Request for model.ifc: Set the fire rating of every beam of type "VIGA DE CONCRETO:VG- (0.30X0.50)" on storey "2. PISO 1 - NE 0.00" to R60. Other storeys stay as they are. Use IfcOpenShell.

First a look at what the model holds.

```python
import ifcopenshell
import ifcopenshell.util.element

model = ifcopenshell.open("model.ifc")
print(model.schema)
storey = next(s for s in model.by_type("IfcBuildingStorey") if s.Name == "2. PISO 1 - NE 0.00")
beams = [e for e in ifcopenshell.util.element.get_decomposition(storey) if e.is_a("IfcBeam")]
seen = {}
for e in beams:
    element_type = ifcopenshell.util.element.get_type(e)
    key = (element_type.Name if element_type != e and element_type else None, ifcopenshell.util.element.get_pset(e, "Pset_BeamCommon", "FireRating"))
    seen[key] = seen.get(key, 0) + 1
for (name, value), count in sorted(seen.items(), key=str):
    print(count, "x", name, "|", value)
```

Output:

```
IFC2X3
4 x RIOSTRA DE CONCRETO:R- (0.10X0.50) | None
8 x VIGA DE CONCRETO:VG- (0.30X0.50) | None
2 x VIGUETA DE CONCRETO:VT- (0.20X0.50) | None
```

```python
import ifcopenshell
import ifcopenshell.api.pset
import ifcopenshell.util.element

model = ifcopenshell.open("model.ifc")

storey = next(s for s in model.by_type("IfcBuildingStorey") if s.Name == "2. PISO 1 - NE 0.00")
beams = [e for e in ifcopenshell.util.element.get_decomposition(storey) if e.is_a("IfcBeam")]

count = 0
for e in beams:
    element_type = ifcopenshell.util.element.get_type(e)
    if element_type in (None, e) or element_type.Name != "VIGA DE CONCRETO:VG- (0.30X0.50)":
        continue
    # add_pset returns the element's existing set when there is one.
    pset = ifcopenshell.api.pset.add_pset(model, product=e, name="Pset_BeamCommon")
    ifcopenshell.api.pset.edit_pset(model, pset=pset, properties={"FireRating": "R60"})
    count += 1

print(count, "beams updated")

model.write("model_v2.ifc")
```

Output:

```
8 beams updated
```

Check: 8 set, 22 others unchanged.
